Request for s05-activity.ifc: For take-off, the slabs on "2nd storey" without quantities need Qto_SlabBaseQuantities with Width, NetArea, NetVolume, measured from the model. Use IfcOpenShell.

First a look at what the model holds.

```python
import ifcopenshell
import ifcopenshell.util.element
import ifcopenshell.util.unit

model = ifcopenshell.open("s05-activity.ifc")
print(model.schema)
for unit_type in ("LENGTHUNIT", "AREAUNIT", "VOLUMEUNIT"):
    print(unit_type, ifcopenshell.util.unit.calculate_unit_scale(model, unit_type))
storey = next(s for s in model.by_type("IfcBuildingStorey") if s.Name == "2nd storey")
slabs = [e for e in ifcopenshell.util.element.get_decomposition(storey) if e.is_a("IfcSlab")]
for e in sorted(slabs, key=lambda e: e.id()):
    print(e.id(), e.is_a(), e.Name, list(ifcopenshell.util.element.get_psets(e, qtos_only=True)), sep=" | ")
```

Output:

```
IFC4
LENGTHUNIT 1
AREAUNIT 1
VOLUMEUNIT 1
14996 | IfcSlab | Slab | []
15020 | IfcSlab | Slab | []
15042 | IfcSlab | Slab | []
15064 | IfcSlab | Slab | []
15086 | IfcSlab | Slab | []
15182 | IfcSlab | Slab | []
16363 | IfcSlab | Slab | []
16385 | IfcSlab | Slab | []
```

```python
import ifcopenshell
import ifcopenshell.api.pset
import ifcopenshell.geom
import ifcopenshell.util.element
import ifcopenshell.util.shape
import ifcopenshell.util.unit

model = ifcopenshell.open("s05-activity.ifc")
unit_scale = ifcopenshell.util.unit.calculate_unit_scale(model)
area_scale = ifcopenshell.util.unit.calculate_unit_scale(model, "AREAUNIT")
volume_scale = ifcopenshell.util.unit.calculate_unit_scale(model, "VOLUMEUNIT")
settings = ifcopenshell.geom.settings()

storey = next(s for s in model.by_type("IfcBuildingStorey") if s.Name == "2nd storey")
slabs = [e for e in ifcopenshell.util.element.get_decomposition(storey) if e.is_a("IfcSlab")]

for e in sorted(slabs, key=lambda e: e.id()):
    if ifcopenshell.util.element.get_psets(e, qtos_only=True, should_inherit=False):
        continue
    # Geometry comes back in metres, in the element's own axes.
    shape = ifcopenshell.geom.create_shape(settings, e)
    values = {
        "Width": ifcopenshell.util.shape.get_z(shape.geometry) / unit_scale,
        "NetArea": ifcopenshell.util.shape.get_footprint_area(shape.geometry) / area_scale,
        "NetVolume": ifcopenshell.util.shape.get_volume(shape.geometry) / volume_scale,
    }
    qto = ifcopenshell.api.pset.add_qto(model, product=e, name="Qto_SlabBaseQuantities")
    ifcopenshell.api.pset.edit_qto(model, qto=qto, properties=values)
    print(e.id(), {k: round(v, 3) for k, v in values.items()})

model.write("s05-activity_v2.ifc")
```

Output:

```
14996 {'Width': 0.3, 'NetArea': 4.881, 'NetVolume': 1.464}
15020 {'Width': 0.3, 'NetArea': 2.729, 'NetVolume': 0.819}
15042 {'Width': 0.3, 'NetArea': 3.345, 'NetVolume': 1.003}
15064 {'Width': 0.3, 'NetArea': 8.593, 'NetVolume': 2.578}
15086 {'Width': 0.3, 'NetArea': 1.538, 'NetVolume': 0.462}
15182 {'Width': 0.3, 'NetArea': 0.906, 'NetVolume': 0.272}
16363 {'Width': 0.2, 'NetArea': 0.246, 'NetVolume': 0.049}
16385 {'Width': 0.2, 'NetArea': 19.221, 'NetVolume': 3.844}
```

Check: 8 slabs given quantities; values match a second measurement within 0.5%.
